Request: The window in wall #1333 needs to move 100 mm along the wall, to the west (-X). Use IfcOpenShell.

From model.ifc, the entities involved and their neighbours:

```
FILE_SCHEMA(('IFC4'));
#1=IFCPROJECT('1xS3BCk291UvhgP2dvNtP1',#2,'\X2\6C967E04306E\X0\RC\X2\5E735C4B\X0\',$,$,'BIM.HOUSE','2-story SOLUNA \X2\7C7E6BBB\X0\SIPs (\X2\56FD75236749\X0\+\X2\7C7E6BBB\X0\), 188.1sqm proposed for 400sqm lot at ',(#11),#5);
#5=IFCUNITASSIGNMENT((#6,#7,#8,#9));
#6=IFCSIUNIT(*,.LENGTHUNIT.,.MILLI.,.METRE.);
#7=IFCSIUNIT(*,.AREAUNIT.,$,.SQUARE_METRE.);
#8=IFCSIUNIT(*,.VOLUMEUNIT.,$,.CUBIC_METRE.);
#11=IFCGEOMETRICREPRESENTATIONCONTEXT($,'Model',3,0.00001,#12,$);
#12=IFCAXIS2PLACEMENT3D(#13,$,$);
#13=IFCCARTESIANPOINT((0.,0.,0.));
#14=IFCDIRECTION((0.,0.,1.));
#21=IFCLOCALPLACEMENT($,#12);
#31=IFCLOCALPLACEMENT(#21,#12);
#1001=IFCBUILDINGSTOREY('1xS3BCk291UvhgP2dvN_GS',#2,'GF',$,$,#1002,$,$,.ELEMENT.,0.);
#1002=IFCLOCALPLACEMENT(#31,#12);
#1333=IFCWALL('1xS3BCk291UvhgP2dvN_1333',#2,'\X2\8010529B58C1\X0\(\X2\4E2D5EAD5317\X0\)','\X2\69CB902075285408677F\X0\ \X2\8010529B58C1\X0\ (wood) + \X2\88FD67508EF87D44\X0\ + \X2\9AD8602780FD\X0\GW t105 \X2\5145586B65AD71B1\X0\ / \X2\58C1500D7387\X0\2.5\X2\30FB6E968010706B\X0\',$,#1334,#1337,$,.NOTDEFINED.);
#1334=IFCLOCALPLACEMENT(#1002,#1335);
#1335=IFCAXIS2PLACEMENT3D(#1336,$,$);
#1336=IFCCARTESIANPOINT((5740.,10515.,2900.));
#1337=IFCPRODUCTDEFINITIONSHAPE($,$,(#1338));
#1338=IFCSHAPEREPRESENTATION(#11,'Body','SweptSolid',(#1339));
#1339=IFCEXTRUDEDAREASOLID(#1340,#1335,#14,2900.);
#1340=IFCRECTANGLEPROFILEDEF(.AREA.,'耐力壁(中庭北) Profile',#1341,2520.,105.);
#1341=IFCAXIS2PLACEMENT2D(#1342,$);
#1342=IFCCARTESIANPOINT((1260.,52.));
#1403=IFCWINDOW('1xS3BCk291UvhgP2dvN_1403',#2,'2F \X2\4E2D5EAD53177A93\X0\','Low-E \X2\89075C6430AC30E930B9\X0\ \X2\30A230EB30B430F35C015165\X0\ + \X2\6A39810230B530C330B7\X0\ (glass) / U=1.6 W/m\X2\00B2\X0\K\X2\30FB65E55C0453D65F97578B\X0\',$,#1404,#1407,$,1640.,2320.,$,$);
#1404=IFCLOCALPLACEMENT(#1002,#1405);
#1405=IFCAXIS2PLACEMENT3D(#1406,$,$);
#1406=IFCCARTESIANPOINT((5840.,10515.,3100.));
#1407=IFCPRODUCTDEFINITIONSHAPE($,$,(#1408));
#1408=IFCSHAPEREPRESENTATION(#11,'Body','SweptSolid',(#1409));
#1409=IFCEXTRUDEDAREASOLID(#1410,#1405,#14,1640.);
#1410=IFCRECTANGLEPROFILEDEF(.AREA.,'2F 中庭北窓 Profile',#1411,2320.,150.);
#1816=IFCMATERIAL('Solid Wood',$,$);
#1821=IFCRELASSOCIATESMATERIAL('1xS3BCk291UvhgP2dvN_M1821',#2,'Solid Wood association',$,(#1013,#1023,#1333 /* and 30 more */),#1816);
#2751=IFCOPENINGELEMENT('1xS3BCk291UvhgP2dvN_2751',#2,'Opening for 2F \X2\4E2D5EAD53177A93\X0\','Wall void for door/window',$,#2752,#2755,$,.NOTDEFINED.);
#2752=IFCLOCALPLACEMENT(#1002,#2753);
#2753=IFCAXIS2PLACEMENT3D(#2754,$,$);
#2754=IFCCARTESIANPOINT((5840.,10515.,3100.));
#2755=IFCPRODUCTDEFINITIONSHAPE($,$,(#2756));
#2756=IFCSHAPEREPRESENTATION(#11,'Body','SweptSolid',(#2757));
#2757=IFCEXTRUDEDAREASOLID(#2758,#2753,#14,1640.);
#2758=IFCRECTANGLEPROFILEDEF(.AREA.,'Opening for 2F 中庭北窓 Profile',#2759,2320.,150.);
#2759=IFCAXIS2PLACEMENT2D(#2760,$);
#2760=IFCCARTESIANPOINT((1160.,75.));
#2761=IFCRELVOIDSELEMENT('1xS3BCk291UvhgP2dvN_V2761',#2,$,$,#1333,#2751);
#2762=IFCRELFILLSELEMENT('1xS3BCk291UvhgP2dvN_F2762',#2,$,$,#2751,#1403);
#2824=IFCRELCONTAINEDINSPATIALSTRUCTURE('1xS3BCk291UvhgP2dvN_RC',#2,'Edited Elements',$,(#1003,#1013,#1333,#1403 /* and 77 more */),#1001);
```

```python
import ifcopenshell
import ifcopenshell.api.geometry
import ifcopenshell.util.placement
import ifcopenshell.util.unit

model = ifcopenshell.open("model.ifc")
unit_scale = ifcopenshell.util.unit.calculate_unit_scale(model)

window = model.by_guid("1xS3BCk291UvhgP2dvN_1403")
opening = window.FillsVoids[0].RelatingOpeningElement
wall = opening.VoidsElements[0].RelatingBuildingElement

wall_matrix = ifcopenshell.util.placement.get_local_placement(wall.ObjectPlacement)
shift = wall_matrix[:3, 0] * -0.1 / unit_scale
before = ifcopenshell.util.placement.get_local_placement(window.ObjectPlacement)[:3, 3].copy()

# The window is not placed relative to its opening, so move both.
for product in (opening, window):
    matrix = ifcopenshell.util.placement.get_local_placement(product.ObjectPlacement)
    matrix[:3, 3] += shift
    ifcopenshell.api.geometry.edit_object_placement(model, product=product, matrix=matrix, is_si=False)

after = ifcopenshell.util.placement.get_local_placement(window.ObjectPlacement)[:3, 3]
print("window moved by", (after - before).round(3) + 0.0)

model.write("model_rev.ifc")
```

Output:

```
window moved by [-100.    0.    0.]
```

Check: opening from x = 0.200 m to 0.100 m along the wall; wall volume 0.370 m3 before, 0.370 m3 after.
